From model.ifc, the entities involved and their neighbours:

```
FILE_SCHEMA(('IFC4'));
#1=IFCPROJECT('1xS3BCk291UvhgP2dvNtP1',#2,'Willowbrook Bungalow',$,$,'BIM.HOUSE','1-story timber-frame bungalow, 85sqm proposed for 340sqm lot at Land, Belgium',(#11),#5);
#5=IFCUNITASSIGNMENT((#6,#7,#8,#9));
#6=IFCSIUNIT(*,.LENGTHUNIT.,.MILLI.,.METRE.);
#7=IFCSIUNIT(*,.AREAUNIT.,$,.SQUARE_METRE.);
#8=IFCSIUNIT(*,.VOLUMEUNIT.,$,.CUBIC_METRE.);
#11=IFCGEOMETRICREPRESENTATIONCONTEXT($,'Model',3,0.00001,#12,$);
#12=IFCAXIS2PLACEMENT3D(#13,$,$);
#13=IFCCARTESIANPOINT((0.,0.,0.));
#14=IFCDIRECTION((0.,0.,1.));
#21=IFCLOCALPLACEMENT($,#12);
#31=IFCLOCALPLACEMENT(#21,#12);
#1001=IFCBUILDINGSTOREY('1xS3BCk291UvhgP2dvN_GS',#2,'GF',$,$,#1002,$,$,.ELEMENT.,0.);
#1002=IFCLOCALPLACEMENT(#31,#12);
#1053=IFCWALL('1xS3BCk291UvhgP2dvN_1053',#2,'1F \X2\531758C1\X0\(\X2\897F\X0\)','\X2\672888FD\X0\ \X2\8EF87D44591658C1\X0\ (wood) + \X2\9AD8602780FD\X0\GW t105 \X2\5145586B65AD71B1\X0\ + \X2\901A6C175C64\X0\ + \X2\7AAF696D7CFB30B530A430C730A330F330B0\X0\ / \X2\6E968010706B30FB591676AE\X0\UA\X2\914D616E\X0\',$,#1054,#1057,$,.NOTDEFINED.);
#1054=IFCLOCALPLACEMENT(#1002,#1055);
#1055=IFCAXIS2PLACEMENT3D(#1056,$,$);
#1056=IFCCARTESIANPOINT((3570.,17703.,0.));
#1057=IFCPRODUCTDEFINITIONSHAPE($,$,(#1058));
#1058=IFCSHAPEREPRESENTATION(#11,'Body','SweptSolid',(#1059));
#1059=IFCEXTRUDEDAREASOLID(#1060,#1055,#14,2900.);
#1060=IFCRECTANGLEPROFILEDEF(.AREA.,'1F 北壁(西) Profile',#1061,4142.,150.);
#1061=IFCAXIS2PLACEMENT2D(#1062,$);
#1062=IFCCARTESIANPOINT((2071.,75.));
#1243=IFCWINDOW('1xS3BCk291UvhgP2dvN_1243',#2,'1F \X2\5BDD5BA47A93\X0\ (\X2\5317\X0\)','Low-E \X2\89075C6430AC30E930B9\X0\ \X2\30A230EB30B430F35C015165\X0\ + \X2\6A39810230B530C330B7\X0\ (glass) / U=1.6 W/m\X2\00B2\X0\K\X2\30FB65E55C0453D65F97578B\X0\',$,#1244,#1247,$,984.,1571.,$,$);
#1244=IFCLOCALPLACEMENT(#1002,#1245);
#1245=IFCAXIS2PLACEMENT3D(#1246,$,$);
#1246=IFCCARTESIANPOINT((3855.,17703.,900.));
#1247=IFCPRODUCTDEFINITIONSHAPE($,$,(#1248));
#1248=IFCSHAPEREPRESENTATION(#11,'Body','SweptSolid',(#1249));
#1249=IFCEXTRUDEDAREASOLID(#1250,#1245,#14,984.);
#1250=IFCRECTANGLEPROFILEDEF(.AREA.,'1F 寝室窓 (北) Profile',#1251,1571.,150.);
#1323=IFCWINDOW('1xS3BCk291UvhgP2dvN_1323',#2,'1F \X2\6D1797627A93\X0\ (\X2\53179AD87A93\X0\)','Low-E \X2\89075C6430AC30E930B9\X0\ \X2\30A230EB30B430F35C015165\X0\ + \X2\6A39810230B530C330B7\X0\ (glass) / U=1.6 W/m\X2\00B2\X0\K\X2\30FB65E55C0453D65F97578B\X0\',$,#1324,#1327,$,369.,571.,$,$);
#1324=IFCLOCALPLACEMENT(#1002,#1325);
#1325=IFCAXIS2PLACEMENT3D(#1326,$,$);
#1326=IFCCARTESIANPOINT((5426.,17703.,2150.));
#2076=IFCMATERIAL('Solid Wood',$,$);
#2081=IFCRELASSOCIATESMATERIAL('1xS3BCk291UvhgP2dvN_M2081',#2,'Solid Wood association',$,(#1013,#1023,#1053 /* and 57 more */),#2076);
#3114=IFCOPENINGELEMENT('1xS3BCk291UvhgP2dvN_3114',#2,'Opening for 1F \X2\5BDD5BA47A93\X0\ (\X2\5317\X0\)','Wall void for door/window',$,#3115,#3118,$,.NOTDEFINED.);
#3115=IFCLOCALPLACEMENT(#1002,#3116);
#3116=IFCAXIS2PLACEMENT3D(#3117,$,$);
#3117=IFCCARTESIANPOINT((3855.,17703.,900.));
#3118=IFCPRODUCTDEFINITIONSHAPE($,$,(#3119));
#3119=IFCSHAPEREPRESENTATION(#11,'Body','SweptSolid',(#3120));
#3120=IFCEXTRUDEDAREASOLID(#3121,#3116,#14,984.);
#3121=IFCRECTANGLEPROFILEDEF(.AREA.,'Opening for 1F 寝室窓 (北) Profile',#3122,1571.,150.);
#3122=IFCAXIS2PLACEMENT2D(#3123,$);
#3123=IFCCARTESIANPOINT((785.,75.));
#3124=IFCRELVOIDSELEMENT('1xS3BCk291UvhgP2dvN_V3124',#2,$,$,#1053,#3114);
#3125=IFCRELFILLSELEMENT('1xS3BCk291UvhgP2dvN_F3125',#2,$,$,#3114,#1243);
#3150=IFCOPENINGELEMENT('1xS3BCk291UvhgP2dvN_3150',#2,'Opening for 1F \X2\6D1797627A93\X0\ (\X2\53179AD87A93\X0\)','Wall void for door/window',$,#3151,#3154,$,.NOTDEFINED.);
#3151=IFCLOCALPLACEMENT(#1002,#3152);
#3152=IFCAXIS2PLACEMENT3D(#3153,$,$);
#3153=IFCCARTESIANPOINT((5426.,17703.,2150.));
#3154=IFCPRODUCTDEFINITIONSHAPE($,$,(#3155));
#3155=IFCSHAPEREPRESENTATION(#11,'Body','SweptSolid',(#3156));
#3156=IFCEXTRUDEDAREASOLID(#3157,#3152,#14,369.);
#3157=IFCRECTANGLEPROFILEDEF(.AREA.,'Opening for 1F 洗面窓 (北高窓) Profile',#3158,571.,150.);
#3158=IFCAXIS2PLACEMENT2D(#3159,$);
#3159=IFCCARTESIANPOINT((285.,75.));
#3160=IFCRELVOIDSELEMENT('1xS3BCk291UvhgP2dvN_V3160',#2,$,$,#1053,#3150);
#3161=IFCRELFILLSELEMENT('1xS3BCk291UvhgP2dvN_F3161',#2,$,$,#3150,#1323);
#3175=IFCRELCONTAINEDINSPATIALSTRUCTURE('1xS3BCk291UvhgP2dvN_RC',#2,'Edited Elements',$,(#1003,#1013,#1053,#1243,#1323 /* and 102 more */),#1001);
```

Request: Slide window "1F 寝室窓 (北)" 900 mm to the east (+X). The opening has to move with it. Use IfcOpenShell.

```python
import ifcopenshell
import ifcopenshell.api.geometry
import ifcopenshell.util.placement
import ifcopenshell.util.unit

model = ifcopenshell.open("model.ifc")
unit_scale = ifcopenshell.util.unit.calculate_unit_scale(model)

window = model.by_guid("1xS3BCk291UvhgP2dvN_1243")
opening = window.FillsVoids[0].RelatingOpeningElement
wall = opening.VoidsElements[0].RelatingBuildingElement

wall_matrix = ifcopenshell.util.placement.get_local_placement(wall.ObjectPlacement)
shift = wall_matrix[:3, 0] * 0.9 / unit_scale
before = ifcopenshell.util.placement.get_local_placement(window.ObjectPlacement)[:3, 3].copy()

# The window is not placed relative to its opening, so move both.
for product in (opening, window):
    matrix = ifcopenshell.util.placement.get_local_placement(product.ObjectPlacement)
    matrix[:3, 3] += shift
    ifcopenshell.api.geometry.edit_object_placement(model, product=product, matrix=matrix, is_si=False)

after = ifcopenshell.util.placement.get_local_placement(window.ObjectPlacement)[:3, 3]
print("window moved by", (after - before).round(3) + 0.0)

model.write("model-out.ifc")
```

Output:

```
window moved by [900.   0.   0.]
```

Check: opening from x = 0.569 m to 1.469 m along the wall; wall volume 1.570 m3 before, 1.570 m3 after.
